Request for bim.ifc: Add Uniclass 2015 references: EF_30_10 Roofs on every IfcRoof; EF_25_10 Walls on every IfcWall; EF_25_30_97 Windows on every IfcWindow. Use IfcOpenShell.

First a look at what the model holds.

```python
import ifcopenshell

model = ifcopenshell.open("bim.ifc")
print(model.schema)
print("classifications:", [c.Name for c in model.by_type("IfcClassification")])
for ifc_class in ("IfcDoor", "IfcRoof", "IfcStair", "IfcWall", "IfcWindow"):
    print(ifc_class, len(model.by_type(ifc_class)))
```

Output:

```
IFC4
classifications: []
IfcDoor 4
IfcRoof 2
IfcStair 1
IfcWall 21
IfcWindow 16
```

```python
import ifcopenshell
import ifcopenshell.api.classification

model = ifcopenshell.open("bim.ifc")

system = ifcopenshell.api.classification.add_classification(model, classification="Uniclass 2015")

codes = {
    "IfcRoof": ("EF_30_10", "Roofs"),
    "IfcWall": ("EF_25_10", "Walls"),
    "IfcWindow": ("EF_25_30_97", "Windows"),
}
for ifc_class, (code, name) in codes.items():
    products = model.by_type(ifc_class)
    ifcopenshell.api.classification.add_reference(
        model, products=products, classification=system, identification=code, name=name
    )
    print(code, len(products))

model.write("bim_edited.ifc")
```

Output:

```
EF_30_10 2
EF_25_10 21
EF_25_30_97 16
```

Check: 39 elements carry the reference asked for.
